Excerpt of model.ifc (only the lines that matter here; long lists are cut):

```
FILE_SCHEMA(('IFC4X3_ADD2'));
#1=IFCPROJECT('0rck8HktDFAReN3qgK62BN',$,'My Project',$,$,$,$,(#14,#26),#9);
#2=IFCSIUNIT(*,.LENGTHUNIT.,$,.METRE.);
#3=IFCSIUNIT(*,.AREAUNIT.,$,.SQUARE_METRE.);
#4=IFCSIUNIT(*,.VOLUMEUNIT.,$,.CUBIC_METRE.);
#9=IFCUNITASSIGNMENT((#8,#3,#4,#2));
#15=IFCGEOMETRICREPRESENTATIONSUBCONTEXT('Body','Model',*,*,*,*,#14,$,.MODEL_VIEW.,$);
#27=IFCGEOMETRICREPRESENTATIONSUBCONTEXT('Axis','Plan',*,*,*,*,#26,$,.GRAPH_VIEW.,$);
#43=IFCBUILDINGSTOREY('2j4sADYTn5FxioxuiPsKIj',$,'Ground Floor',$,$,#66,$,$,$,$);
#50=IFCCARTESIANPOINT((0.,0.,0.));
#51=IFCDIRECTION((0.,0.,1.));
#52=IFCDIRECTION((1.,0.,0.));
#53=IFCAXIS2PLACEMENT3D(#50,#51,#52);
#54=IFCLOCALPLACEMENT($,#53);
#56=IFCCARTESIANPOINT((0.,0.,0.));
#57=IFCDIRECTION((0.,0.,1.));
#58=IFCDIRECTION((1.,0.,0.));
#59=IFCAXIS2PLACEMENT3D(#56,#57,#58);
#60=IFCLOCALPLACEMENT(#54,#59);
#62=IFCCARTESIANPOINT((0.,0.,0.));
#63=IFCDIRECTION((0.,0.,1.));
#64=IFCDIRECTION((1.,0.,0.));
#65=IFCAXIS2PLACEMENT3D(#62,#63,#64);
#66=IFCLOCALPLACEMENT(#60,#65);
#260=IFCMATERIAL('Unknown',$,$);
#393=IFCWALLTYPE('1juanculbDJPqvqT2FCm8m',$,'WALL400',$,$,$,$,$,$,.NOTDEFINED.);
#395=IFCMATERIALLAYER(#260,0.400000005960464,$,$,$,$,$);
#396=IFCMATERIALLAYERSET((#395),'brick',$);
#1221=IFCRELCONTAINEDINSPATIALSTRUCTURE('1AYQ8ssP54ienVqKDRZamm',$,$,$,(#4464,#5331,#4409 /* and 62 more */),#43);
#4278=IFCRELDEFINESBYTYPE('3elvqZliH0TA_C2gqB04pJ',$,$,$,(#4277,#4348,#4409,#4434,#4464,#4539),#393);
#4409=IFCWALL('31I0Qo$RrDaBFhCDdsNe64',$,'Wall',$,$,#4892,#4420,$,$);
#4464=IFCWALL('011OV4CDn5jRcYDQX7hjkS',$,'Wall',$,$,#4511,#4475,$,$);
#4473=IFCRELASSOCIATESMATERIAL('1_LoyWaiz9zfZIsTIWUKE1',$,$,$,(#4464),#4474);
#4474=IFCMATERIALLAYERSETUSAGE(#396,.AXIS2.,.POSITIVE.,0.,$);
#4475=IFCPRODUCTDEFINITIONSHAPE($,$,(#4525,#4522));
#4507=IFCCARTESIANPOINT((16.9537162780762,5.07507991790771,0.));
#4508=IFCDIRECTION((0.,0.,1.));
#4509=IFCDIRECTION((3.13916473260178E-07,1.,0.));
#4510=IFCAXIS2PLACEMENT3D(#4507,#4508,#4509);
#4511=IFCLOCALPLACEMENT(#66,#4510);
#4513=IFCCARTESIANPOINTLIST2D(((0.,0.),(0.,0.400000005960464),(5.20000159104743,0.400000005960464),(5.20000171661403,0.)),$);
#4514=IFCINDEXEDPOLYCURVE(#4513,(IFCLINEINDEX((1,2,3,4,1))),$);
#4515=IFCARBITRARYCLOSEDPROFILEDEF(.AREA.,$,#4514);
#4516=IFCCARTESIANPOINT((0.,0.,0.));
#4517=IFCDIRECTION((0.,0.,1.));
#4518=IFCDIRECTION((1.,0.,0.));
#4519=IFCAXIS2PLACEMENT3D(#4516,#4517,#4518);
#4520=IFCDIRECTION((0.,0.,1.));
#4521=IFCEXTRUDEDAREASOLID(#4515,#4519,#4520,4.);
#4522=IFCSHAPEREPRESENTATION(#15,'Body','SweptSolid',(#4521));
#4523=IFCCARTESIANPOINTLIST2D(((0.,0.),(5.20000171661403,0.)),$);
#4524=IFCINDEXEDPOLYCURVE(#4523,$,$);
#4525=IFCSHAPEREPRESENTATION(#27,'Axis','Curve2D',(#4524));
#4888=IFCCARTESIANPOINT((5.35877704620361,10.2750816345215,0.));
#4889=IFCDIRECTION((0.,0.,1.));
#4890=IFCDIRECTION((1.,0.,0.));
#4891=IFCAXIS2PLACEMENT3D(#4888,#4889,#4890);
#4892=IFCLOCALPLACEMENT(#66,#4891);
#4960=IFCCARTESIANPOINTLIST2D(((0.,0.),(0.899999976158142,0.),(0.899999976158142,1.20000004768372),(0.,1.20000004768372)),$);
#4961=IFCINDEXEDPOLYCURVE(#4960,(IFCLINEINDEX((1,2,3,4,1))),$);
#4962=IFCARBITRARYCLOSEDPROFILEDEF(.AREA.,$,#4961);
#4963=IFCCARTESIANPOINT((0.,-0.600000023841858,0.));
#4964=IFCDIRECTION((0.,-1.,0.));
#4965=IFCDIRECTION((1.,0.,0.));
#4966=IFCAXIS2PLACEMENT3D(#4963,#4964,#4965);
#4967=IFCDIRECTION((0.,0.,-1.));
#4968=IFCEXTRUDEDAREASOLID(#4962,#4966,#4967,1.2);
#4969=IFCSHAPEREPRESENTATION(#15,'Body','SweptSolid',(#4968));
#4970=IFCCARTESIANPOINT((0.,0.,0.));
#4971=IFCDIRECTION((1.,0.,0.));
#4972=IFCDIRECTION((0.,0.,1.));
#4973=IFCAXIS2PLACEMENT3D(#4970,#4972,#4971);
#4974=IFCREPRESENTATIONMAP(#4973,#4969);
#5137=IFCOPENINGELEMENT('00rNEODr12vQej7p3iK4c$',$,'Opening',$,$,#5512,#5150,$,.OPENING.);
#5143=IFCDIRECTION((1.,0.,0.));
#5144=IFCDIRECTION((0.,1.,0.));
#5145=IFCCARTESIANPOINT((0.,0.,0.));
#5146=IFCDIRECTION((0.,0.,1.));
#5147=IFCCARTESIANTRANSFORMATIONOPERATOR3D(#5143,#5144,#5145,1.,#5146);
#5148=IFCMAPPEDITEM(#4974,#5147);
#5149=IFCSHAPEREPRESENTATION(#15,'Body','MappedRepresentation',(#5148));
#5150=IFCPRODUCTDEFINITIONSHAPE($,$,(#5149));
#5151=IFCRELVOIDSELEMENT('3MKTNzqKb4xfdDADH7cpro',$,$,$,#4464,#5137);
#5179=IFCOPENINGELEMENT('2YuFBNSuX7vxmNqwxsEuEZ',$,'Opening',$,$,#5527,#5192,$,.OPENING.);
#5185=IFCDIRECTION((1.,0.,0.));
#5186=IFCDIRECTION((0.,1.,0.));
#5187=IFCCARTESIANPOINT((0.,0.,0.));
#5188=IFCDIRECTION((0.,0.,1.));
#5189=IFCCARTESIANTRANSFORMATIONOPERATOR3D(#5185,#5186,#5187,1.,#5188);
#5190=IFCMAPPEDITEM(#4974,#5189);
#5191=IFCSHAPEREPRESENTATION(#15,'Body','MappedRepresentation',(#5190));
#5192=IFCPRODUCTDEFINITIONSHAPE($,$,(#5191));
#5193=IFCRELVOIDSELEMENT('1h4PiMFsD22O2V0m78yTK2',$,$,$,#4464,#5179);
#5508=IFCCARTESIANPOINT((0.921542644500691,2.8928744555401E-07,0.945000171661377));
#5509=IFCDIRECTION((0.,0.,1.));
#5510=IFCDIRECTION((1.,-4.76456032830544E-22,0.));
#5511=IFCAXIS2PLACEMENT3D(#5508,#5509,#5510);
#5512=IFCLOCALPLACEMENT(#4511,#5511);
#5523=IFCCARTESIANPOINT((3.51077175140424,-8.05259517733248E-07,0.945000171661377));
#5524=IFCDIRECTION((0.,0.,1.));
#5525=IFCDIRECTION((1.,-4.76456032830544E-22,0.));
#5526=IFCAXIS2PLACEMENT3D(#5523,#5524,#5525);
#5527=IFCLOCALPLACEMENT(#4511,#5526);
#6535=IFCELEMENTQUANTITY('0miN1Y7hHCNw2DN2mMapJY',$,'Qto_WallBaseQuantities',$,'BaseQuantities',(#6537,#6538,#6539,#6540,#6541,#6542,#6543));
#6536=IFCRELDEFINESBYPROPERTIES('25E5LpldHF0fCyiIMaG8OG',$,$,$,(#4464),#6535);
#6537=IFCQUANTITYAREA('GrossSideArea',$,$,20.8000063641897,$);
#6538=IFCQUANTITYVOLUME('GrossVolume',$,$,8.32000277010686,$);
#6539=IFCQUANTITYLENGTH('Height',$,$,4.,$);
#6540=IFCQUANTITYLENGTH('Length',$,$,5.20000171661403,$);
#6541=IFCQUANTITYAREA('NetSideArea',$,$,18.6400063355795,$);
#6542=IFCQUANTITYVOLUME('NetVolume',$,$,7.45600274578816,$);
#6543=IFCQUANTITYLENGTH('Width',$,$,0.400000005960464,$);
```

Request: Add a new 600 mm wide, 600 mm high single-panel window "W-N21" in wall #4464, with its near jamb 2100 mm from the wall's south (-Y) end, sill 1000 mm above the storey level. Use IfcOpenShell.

```python
import numpy as np
import ifcopenshell
import ifcopenshell.api.feature
import ifcopenshell.api.geometry
import ifcopenshell.api.pset
import ifcopenshell.api.root
import ifcopenshell.api.spatial
import ifcopenshell.geom
import ifcopenshell.util.element
import ifcopenshell.util.placement
import ifcopenshell.util.representation
import ifcopenshell.util.shape
import ifcopenshell.util.unit

model = ifcopenshell.open("model.ifc")
unit_scale = ifcopenshell.util.unit.calculate_unit_scale(model)
area_scale = ifcopenshell.util.unit.calculate_unit_scale(model, "AREAUNIT")
volume_scale = ifcopenshell.util.unit.calculate_unit_scale(model, "VOLUMEUNIT")
settings = ifcopenshell.geom.settings()


def volume(element):
    """Net volume in cubic metres, openings subtracted."""
    shape = ifcopenshell.geom.create_shape(settings, element)
    return ifcopenshell.util.shape.get_volume(shape.geometry)


wall = model.by_guid("011OV4CDn5jRcYDQX7hjkS")
storey = ifcopenshell.util.element.get_container(wall, ifc_class="IfcBuildingStorey")
context = ifcopenshell.util.representation.get_context(model, "Model", "Body", "MODEL_VIEW")
before = volume(wall)

width, height, from_end, sill = 0.6, 0.6, 2.1, 1  # metres

# The wall runs along its own X axis, and the end named is its -X end.
wall_shape = ifcopenshell.geom.create_shape(settings, wall)
x, y, z = ifcopenshell.util.shape.get_vertices(wall_shape.geometry).T
start = x.min() + from_end
face, thickness = float(y.min()), float(y.max() - y.min())
wall_matrix = ifcopenshell.util.placement.get_local_placement(wall.ObjectPlacement)
level = ifcopenshell.util.placement.get_local_placement(storey.ObjectPlacement)[2, 3]


def in_wall(x, y):
    """Placement at x, y metres in the wall's axes, at sill height."""
    matrix = wall_matrix.copy()
    matrix[:, 3] = wall_matrix @ np.array([x / unit_scale, y / unit_scale, 0.0, 1.0])
    matrix[2, 3] = level + sill / unit_scale
    return matrix


# Opening: a box that overshoots both wall faces by 50 mm.
opening = ifcopenshell.api.root.create_entity(model, ifc_class="IfcOpeningElement", predefined_type="OPENING")
box = ifcopenshell.api.geometry.add_wall_representation(
    model, context=context, length=width, height=height, thickness=thickness + 0.1
)
ifcopenshell.api.geometry.assign_representation(model, product=opening, representation=box)
ifcopenshell.api.geometry.edit_object_placement(model, product=opening, matrix=in_wall(start, face - 0.05), is_si=False)
ifcopenshell.api.feature.add_feature(model, feature=opening, element=wall)

window = ifcopenshell.api.root.create_entity(model, ifc_class="IfcWindow", name="W-N21", predefined_type="WINDOW")
window.OverallWidth, window.OverallHeight = width / unit_scale, height / unit_scale
window.PartitioningType = "SINGLE_PANEL"
body = ifcopenshell.api.geometry.add_window_representation(
    model,
    context=context,
    overall_width=window.OverallWidth,
    overall_height=window.OverallHeight,
    partition_type="SINGLE_PANEL",
)
ifcopenshell.api.geometry.assign_representation(model, product=window, representation=body)
ifcopenshell.api.spatial.assign_container(model, products=[window], relating_structure=storey)
ifcopenshell.api.feature.add_filling(model, opening=opening, element=window)

# Centre the window in the wall's thickness.
ifcopenshell.api.geometry.edit_object_placement(model, product=window, matrix=in_wall(start, face), is_si=False)
window_shape = ifcopenshell.geom.create_shape(settings, window)
depth = ifcopenshell.util.shape.get_vertices(window_shape.geometry)[:, 1]
offset = face + thickness / 2 - (depth.min() + depth.max()) / 2
ifcopenshell.api.geometry.edit_object_placement(model, product=window, matrix=in_wall(start, offset), is_si=False)

after = volume(wall)

# Update the wall's stored quantities.
qto = model.by_id(ifcopenshell.util.element.get_pset(wall, "Qto_WallBaseQuantities", should_inherit=False)["id"])
ifcopenshell.api.pset.edit_qto(model, qto=qto, properties={
    "NetSideArea": after / thickness / area_scale,
    "NetVolume": after / volume_scale,
})

print(f"wall volume {before:.3f} -> {after:.3f} m3")

model.write("model_rev.ifc")
```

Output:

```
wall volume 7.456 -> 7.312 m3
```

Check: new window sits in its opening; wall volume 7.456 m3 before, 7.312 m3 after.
